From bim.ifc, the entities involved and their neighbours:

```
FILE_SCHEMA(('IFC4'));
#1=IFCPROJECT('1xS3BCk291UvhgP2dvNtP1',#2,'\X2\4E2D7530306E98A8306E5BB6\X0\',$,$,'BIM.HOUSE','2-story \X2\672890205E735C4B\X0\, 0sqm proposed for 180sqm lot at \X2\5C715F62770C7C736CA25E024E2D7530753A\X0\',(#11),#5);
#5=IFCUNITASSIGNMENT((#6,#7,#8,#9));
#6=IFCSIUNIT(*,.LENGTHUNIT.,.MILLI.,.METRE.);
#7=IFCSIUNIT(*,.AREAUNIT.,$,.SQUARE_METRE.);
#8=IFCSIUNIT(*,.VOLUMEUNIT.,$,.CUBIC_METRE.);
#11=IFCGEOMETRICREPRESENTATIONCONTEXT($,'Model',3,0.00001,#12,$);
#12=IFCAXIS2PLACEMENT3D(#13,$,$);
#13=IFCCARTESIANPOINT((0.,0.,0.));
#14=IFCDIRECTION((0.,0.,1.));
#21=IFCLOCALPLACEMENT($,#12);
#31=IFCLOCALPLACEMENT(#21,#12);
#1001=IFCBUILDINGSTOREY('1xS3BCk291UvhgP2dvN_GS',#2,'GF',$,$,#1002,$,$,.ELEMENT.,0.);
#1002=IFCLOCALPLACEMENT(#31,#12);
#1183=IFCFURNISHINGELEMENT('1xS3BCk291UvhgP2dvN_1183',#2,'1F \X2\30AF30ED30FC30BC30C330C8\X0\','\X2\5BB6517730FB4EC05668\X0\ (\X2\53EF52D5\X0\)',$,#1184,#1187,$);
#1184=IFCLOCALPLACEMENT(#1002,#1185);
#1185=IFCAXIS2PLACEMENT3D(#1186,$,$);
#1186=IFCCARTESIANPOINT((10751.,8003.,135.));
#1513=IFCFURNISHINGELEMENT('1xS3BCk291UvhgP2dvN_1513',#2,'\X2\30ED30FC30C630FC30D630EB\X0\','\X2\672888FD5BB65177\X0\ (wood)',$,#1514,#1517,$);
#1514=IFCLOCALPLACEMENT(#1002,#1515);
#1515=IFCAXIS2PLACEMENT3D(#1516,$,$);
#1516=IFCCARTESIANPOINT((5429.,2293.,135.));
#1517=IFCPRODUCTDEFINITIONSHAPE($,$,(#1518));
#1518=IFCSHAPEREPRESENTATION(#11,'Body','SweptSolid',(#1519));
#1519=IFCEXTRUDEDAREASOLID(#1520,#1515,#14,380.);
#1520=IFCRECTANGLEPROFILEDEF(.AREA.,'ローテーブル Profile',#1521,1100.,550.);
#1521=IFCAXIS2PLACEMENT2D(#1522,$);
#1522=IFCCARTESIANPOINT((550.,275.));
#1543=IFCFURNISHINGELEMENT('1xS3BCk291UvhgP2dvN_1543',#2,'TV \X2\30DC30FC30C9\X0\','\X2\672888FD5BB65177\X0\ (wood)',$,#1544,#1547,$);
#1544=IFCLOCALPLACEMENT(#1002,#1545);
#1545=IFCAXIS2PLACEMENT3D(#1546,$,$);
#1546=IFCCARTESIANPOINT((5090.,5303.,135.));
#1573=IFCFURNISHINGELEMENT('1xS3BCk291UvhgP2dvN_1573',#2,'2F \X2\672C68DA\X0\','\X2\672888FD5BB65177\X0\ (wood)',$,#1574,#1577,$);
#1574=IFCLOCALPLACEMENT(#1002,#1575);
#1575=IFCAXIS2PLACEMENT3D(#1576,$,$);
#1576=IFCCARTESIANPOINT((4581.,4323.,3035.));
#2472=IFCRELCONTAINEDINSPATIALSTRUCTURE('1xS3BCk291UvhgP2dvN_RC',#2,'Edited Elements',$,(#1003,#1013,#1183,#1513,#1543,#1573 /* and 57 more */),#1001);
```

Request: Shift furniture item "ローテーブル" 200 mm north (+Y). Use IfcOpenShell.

```python
import ifcopenshell
import ifcopenshell.api.geometry
import ifcopenshell.util.placement

model = ifcopenshell.open("bim.ifc")

item = model.by_guid("1xS3BCk291UvhgP2dvN_1513")
matrix = ifcopenshell.util.placement.get_local_placement(item.ObjectPlacement)
matrix[1, 3] += 200.0
ifcopenshell.api.geometry.edit_object_placement(model, product=item, matrix=matrix, is_si=False)

print(ifcopenshell.util.placement.get_local_placement(item.ObjectPlacement).round(3) + 0.0)

model.write("bim_rev.ifc")
```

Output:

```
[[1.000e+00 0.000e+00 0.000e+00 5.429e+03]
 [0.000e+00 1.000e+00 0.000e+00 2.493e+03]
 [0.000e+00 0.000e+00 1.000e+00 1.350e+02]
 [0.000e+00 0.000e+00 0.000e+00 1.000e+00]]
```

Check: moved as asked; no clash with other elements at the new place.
